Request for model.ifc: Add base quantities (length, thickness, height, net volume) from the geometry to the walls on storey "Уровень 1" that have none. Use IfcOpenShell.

First a look at what the model holds.

```python
import ifcopenshell
import ifcopenshell.util.element
import ifcopenshell.util.unit

model = ifcopenshell.open("model.ifc")
print(model.schema)
for unit_type in ("LENGTHUNIT", "AREAUNIT", "VOLUMEUNIT"):
    print(unit_type, ifcopenshell.util.unit.calculate_unit_scale(model, unit_type))
storey = next(s for s in model.by_type("IfcBuildingStorey") if s.Name == "Уровень 1")
walls = [e for e in ifcopenshell.util.element.get_decomposition(storey) if e.is_a("IfcWall")]
for e in sorted(walls, key=lambda e: e.id()):
    print(e.id(), e.is_a(), e.Name, list(ifcopenshell.util.element.get_psets(e, qtos_only=True)), sep=" | ")
```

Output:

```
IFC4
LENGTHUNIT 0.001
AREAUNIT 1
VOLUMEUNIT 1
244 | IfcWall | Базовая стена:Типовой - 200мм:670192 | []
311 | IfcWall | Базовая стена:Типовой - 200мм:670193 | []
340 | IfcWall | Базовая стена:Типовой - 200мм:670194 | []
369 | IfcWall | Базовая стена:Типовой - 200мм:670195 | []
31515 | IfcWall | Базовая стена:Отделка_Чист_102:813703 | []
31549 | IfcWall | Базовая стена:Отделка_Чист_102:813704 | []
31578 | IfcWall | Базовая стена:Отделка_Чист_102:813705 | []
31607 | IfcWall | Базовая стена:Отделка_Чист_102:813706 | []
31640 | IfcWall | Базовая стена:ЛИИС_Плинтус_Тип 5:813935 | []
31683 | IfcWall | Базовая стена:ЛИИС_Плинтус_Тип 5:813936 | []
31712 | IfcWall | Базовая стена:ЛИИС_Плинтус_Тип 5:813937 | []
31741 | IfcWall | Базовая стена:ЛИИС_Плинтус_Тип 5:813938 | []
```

```python
import ifcopenshell
import ifcopenshell.api.pset
import ifcopenshell.geom
import ifcopenshell.util.element
import ifcopenshell.util.shape
import ifcopenshell.util.unit

model = ifcopenshell.open("model.ifc")
unit_scale = ifcopenshell.util.unit.calculate_unit_scale(model)
volume_scale = ifcopenshell.util.unit.calculate_unit_scale(model, "VOLUMEUNIT")
settings = ifcopenshell.geom.settings()

storey = next(s for s in model.by_type("IfcBuildingStorey") if s.Name == "Уровень 1")
walls = [e for e in ifcopenshell.util.element.get_decomposition(storey) if e.is_a("IfcWall")]

for e in sorted(walls, key=lambda e: e.id()):
    if ifcopenshell.util.element.get_psets(e, qtos_only=True, should_inherit=False):
        continue
    # Geometry comes back in metres, in the element's own axes.
    shape = ifcopenshell.geom.create_shape(settings, e)
    values = {
        "Length": ifcopenshell.util.shape.get_x(shape.geometry) / unit_scale,
        "Width": ifcopenshell.util.shape.get_y(shape.geometry) / unit_scale,
        "Height": ifcopenshell.util.shape.get_z(shape.geometry) / unit_scale,
        "NetVolume": ifcopenshell.util.shape.get_volume(shape.geometry) / volume_scale,
    }
    qto = ifcopenshell.api.pset.add_qto(model, product=e, name="Qto_WallBaseQuantities")
    ifcopenshell.api.pset.edit_qto(model, qto=qto, properties=values)
    print(e.id(), {k: round(v, 3) for k, v in values.items()})

model.write("model-out.ifc")
```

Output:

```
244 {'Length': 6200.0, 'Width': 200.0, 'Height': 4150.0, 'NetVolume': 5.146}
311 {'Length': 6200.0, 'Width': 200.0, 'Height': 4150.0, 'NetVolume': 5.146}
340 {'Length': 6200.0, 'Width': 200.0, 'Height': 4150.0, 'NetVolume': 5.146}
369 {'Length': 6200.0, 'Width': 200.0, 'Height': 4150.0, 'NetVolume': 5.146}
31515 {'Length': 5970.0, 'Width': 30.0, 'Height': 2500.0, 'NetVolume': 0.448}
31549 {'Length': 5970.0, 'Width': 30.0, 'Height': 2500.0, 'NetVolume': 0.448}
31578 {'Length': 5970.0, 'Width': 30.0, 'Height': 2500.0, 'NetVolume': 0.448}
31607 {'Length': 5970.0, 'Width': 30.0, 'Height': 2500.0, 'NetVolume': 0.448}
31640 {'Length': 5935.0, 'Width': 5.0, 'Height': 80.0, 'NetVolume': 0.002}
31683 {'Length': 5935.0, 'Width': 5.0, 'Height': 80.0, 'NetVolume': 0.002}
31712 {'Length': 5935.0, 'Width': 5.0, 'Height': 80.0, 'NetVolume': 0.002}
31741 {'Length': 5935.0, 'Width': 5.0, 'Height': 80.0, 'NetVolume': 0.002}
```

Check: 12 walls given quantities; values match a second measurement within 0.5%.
